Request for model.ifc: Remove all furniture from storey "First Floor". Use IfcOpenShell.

First a look at what the model holds.

```python
import ifcopenshell
import ifcopenshell.util.element

model = ifcopenshell.open("model.ifc")
print(model.schema)
storey = next(s for s in model.by_type("IfcBuildingStorey") if s.Name == "First Floor")
furniture = [e for e in ifcopenshell.util.element.get_decomposition(storey) if e.is_a("IfcFurnishingElement")]
seen = {}
for e in furniture:
    element_type = ifcopenshell.util.element.get_type(e)
    name = element_type.Name if element_type not in (None, e) else None
    seen[name] = seen.get(name, 0) + 1
for name, count in sorted(seen.items(), key=str):
    print(count, "x", name)
```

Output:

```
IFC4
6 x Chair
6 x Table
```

```python
import ifcopenshell
import ifcopenshell.api.root
import ifcopenshell.util.element

model = ifcopenshell.open("model.ifc")

storey = next(s for s in model.by_type("IfcBuildingStorey") if s.Name == "First Floor")
furniture = [e for e in ifcopenshell.util.element.get_decomposition(storey) if e.is_a("IfcFurnishingElement")]

for e in furniture:
    ifcopenshell.api.root.remove_product(model, product=e)
print(len(furniture), "removed")

model.write("model_rev.ifc")
```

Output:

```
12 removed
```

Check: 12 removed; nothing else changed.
